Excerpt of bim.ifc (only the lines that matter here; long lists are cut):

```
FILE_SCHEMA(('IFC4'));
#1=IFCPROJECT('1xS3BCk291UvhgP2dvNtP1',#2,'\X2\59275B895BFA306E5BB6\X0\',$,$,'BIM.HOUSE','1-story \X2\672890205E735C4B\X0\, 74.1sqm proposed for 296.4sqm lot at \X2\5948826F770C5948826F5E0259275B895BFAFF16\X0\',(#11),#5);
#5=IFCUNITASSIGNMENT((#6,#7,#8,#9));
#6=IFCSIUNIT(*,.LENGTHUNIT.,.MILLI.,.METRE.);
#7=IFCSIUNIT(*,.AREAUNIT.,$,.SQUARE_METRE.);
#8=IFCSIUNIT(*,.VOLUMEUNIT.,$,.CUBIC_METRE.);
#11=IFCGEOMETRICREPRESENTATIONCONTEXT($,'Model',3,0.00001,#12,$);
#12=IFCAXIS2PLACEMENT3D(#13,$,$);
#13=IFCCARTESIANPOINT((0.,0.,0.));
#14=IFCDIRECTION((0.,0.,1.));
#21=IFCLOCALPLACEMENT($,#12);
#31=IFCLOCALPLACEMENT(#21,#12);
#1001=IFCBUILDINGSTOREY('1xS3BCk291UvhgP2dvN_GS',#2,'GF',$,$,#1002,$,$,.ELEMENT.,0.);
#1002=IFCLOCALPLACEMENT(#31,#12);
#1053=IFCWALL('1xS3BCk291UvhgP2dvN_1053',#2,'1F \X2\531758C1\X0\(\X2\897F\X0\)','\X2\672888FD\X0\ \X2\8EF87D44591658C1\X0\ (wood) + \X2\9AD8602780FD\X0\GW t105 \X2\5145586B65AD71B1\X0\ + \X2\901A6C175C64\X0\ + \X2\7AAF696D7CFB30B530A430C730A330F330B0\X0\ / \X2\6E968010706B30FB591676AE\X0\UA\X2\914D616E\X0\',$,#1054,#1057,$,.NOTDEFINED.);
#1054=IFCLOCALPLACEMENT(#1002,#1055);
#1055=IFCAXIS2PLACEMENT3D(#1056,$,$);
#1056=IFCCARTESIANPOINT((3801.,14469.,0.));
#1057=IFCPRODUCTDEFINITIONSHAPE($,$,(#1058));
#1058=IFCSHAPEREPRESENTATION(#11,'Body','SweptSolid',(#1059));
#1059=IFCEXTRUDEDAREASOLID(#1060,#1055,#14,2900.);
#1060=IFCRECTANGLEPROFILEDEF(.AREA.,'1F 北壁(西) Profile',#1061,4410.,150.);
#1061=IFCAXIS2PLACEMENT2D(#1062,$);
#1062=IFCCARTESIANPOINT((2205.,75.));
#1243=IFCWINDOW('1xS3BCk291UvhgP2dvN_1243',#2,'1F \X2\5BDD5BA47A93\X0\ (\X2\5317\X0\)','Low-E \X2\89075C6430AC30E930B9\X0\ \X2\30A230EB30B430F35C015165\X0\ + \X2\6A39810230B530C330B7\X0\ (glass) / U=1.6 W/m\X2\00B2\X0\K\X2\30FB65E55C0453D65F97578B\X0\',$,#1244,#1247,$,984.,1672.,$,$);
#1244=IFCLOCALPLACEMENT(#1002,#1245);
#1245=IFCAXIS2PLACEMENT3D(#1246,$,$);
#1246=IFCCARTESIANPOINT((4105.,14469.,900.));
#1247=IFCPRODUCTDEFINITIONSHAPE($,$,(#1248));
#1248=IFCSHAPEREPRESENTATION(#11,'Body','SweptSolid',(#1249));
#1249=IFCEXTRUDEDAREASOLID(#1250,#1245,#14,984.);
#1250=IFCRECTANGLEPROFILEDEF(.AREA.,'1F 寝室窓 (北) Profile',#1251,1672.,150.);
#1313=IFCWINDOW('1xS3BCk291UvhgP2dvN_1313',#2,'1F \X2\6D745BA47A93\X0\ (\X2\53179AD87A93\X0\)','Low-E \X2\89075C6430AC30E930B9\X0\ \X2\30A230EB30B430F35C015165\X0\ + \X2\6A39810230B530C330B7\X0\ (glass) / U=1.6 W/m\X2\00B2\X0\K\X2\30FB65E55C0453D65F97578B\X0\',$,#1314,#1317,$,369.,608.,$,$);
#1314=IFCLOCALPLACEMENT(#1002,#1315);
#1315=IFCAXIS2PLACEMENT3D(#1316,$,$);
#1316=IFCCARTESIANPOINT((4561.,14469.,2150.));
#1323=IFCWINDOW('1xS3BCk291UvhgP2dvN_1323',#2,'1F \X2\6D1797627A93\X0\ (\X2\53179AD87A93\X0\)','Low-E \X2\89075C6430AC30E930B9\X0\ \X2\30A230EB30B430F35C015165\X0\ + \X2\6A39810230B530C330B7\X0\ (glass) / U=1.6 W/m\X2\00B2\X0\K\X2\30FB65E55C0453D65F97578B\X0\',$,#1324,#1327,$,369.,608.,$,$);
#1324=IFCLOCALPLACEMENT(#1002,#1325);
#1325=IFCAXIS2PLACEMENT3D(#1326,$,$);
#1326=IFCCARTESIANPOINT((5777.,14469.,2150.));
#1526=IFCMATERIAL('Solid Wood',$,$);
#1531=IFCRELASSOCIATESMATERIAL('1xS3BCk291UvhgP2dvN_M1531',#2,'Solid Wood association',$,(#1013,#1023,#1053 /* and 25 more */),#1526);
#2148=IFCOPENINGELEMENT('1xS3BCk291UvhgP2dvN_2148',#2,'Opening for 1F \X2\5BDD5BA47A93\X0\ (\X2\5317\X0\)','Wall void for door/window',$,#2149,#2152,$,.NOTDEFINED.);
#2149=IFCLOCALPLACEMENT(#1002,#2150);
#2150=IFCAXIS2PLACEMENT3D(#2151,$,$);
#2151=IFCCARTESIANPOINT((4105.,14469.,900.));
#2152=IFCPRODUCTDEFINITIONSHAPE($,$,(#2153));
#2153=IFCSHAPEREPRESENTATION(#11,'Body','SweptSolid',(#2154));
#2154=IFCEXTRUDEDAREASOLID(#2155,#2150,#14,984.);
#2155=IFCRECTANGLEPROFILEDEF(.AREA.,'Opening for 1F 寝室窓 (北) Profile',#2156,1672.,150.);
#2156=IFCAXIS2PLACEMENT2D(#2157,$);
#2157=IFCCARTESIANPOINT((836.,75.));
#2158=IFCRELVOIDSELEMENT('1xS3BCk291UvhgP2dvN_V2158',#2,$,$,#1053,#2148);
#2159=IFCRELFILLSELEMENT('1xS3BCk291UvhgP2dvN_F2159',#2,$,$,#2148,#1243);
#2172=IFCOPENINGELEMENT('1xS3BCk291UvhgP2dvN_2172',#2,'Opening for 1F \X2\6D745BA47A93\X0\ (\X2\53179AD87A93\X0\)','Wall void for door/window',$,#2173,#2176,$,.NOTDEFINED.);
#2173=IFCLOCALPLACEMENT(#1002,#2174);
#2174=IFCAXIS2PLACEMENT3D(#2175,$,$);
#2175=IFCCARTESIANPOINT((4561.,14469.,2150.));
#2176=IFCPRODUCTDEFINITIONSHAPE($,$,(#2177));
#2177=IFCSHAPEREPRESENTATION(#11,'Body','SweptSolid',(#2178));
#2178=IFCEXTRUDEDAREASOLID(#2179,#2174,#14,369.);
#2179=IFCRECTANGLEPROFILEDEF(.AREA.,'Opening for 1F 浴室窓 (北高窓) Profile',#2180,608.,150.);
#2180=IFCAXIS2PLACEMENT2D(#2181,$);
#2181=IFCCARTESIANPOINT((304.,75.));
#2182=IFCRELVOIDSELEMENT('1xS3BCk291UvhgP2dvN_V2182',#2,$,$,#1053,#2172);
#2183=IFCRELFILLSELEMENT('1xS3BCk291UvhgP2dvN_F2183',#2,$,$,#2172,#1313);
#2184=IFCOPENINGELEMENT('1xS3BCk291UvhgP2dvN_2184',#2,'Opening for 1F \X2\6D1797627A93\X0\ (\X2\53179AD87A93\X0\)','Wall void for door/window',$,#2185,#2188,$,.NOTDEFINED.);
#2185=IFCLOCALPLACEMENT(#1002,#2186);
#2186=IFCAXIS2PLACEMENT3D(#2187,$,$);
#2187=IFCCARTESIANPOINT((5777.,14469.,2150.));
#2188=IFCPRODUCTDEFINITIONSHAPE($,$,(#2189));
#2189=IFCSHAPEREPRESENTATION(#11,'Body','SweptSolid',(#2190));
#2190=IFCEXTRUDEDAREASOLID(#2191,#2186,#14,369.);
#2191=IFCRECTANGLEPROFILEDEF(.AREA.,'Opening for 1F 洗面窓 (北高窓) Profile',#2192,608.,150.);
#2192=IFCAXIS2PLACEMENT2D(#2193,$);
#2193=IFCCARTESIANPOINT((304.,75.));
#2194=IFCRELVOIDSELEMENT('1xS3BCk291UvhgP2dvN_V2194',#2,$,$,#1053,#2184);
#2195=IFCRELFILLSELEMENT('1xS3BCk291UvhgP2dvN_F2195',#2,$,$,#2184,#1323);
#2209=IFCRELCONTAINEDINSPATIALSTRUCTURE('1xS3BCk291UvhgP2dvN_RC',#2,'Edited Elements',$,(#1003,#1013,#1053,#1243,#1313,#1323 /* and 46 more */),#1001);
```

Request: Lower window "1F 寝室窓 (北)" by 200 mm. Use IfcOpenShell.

```python
import numpy as np
import ifcopenshell
import ifcopenshell.api.geometry
import ifcopenshell.util.placement
import ifcopenshell.util.unit

model = ifcopenshell.open("bim.ifc")
unit_scale = ifcopenshell.util.unit.calculate_unit_scale(model)

window = model.by_guid("1xS3BCk291UvhgP2dvN_1243")
opening = window.FillsVoids[0].RelatingOpeningElement
dz = -0.2 / unit_scale

shift = np.array([0.0, 0.0, dz])
# The window is not placed relative to its opening, so move both.
for product in (opening, window):
    matrix = ifcopenshell.util.placement.get_local_placement(product.ObjectPlacement)
    matrix[:3, 3] += shift
    ifcopenshell.api.geometry.edit_object_placement(model, product=product, matrix=matrix, is_si=False)

print(f"moved by {dz * unit_scale:+.3f} m")

model.write("bim-out.ifc")
```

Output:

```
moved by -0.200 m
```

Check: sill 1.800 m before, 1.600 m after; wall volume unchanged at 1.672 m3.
